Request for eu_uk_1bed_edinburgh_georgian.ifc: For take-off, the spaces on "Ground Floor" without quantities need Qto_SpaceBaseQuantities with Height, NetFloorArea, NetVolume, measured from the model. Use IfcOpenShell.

First a look at what the model holds.

```python
import ifcopenshell
import ifcopenshell.util.element
import ifcopenshell.util.unit

model = ifcopenshell.open("eu_uk_1bed_edinburgh_georgian.ifc")
print(model.schema)
for unit_type in ("LENGTHUNIT", "AREAUNIT", "VOLUMEUNIT"):
    print(unit_type, ifcopenshell.util.unit.calculate_unit_scale(model, unit_type))
storey = next(s for s in model.by_type("IfcBuildingStorey") if s.Name == "Ground Floor")
spaces = [e for e in ifcopenshell.util.element.get_decomposition(storey) if e.is_a("IfcSpace")]
for e in sorted(spaces, key=lambda e: e.id()):
    print(e.id(), e.is_a(), e.Name, list(ifcopenshell.util.element.get_psets(e, qtos_only=True)), sep=" | ")
```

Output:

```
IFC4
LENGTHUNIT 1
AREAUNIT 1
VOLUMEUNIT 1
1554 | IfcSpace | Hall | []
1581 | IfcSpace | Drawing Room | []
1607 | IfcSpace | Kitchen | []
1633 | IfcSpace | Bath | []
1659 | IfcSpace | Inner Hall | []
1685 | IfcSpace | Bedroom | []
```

```python
import ifcopenshell
import ifcopenshell.api.pset
import ifcopenshell.geom
import ifcopenshell.util.element
import ifcopenshell.util.shape
import ifcopenshell.util.unit

model = ifcopenshell.open("eu_uk_1bed_edinburgh_georgian.ifc")
unit_scale = ifcopenshell.util.unit.calculate_unit_scale(model)
area_scale = ifcopenshell.util.unit.calculate_unit_scale(model, "AREAUNIT")
volume_scale = ifcopenshell.util.unit.calculate_unit_scale(model, "VOLUMEUNIT")
settings = ifcopenshell.geom.settings()

storey = next(s for s in model.by_type("IfcBuildingStorey") if s.Name == "Ground Floor")
spaces = [e for e in ifcopenshell.util.element.get_decomposition(storey) if e.is_a("IfcSpace")]

for e in sorted(spaces, key=lambda e: e.id()):
    if ifcopenshell.util.element.get_psets(e, qtos_only=True, should_inherit=False):
        continue
    # Geometry comes back in metres, in the element's own axes.
    shape = ifcopenshell.geom.create_shape(settings, e)
    values = {
        "Height": ifcopenshell.util.shape.get_z(shape.geometry) / unit_scale,
        "NetFloorArea": ifcopenshell.util.shape.get_footprint_area(shape.geometry) / area_scale,
        "NetVolume": ifcopenshell.util.shape.get_volume(shape.geometry) / volume_scale,
    }
    qto = ifcopenshell.api.pset.add_qto(model, product=e, name="Qto_SpaceBaseQuantities")
    ifcopenshell.api.pset.edit_qto(model, qto=qto, properties=values)
    print(e.id(), {k: round(v, 3) for k, v in values.items()})

model.write("eu_uk_1bed_edinburgh_georgian-out.ifc")
```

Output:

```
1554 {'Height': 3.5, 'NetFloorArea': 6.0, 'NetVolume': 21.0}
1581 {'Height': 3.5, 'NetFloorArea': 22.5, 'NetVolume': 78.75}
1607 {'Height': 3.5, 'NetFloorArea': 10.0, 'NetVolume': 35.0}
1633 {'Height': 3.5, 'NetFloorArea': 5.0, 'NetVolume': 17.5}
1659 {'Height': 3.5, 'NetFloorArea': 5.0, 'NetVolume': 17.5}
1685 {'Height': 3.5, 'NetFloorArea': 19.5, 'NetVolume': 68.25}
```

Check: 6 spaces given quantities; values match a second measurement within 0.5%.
